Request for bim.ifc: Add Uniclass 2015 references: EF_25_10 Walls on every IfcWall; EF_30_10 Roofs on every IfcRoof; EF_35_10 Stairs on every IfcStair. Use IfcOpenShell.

First a look at what the model holds.

```python
import ifcopenshell

model = ifcopenshell.open("bim.ifc")
print(model.schema)
print("classifications:", [c.Name for c in model.by_type("IfcClassification")])
for ifc_class in ("IfcDoor", "IfcRoof", "IfcStair", "IfcWall", "IfcWindow"):
    print(ifc_class, len(model.by_type(ifc_class)))
```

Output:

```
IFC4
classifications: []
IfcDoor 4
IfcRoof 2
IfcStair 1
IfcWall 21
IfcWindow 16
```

```python
import ifcopenshell
import ifcopenshell.api.classification

model = ifcopenshell.open("bim.ifc")

system = ifcopenshell.api.classification.add_classification(model, classification="Uniclass 2015")

codes = {
    "IfcWall": ("EF_25_10", "Walls"),
    "IfcRoof": ("EF_30_10", "Roofs"),
    "IfcStair": ("EF_35_10", "Stairs"),
}
for ifc_class, (code, name) in codes.items():
    products = model.by_type(ifc_class)
    ifcopenshell.api.classification.add_reference(
        model, products=products, classification=system, identification=code, name=name
    )
    print(code, len(products))

model.write("bim_rev.ifc")
```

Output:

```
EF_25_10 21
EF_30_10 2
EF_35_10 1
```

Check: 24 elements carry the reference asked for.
